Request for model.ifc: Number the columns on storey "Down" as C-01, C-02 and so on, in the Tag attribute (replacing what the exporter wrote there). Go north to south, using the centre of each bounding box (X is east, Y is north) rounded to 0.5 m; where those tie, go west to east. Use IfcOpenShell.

First a look at what the model holds.

```python
import ifcopenshell
import ifcopenshell.util.element
import ifcopenshell.util.placement

model = ifcopenshell.open("model.ifc")
print(model.schema)
storey = next(s for s in model.by_type("IfcBuildingStorey") if s.Name == "Down")
columns = [e for e in ifcopenshell.util.element.get_decomposition(storey) if e.is_a("IfcColumn")]
for e in sorted(columns, key=lambda e: e.id()):
    origin = ifcopenshell.util.placement.get_local_placement(e.ObjectPlacement)[:3, 3]
    print(e.id(), e.Tag, e.Name, origin.round(2) + 0.0, sep=" | ")
```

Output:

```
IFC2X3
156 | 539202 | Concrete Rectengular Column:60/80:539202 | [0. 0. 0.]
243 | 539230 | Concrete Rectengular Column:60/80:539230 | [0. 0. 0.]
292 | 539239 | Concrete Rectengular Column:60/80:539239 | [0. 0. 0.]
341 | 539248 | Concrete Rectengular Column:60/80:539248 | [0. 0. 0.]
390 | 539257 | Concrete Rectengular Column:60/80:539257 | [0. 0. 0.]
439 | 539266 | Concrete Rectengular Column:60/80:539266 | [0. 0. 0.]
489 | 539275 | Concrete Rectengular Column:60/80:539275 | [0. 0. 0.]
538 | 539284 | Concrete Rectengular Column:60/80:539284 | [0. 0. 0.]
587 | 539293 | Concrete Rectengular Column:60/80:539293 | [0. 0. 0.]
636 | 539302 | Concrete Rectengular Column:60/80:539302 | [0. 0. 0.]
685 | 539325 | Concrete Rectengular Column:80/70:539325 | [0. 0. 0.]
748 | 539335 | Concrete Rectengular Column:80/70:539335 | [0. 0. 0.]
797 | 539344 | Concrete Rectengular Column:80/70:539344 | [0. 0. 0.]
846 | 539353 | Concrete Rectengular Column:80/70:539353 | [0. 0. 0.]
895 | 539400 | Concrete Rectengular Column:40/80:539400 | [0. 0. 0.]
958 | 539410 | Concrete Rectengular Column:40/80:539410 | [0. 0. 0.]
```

```python
import ifcopenshell
import ifcopenshell.geom
import ifcopenshell.util.element
import ifcopenshell.util.shape

model = ifcopenshell.open("model.ifc")
settings = ifcopenshell.geom.settings()
settings.set("use-world-coords", True)


def centre(element):
    shape = ifcopenshell.geom.create_shape(settings, element)
    return ifcopenshell.util.shape.get_bbox_centroid(shape.geometry)


storey = next(s for s in model.by_type("IfcBuildingStorey") if s.Name == "Down")
columns = [e for e in ifcopenshell.util.element.get_decomposition(storey) if e.is_a("IfcColumn")]

# Insertion points can sit at a corner or the storey origin, so sort by the geometry (in metres).
centres = {e: centre(e) for e in columns}
columns.sort(key=lambda e: (-round(centres[e][1] / 0.5), centres[e][0]))

for i, e in enumerate(columns, start=1):
    number = f"C-{i:02d}"
    e.Tag = number
    print(e.id(), number)

model.write("model_rev.ifc")
```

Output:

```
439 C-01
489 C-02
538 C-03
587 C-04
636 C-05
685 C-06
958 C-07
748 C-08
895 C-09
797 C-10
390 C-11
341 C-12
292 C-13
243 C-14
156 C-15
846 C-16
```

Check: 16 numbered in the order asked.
